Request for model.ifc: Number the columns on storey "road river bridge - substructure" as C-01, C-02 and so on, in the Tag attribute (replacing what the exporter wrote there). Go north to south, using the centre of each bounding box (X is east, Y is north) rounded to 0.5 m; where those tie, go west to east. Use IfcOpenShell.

First a look at what the model holds.

```python
import ifcopenshell
import ifcopenshell.util.element
import ifcopenshell.util.placement

model = ifcopenshell.open("model.ifc")
print(model.schema)
storey = next(s for s in model.by_type("IfcBuildingStorey") if s.Name == "road river bridge - substructure")
columns = [e for e in ifcopenshell.util.element.get_decomposition(storey) if e.is_a("IfcColumn")]
for e in sorted(columns, key=lambda e: e.id()):
    origin = ifcopenshell.util.placement.get_local_placement(e.ObjectPlacement)[:3, 3]
    print(e.id(), e.Tag, e.Name, origin.round(2) + 0.0, sep=" | ")
```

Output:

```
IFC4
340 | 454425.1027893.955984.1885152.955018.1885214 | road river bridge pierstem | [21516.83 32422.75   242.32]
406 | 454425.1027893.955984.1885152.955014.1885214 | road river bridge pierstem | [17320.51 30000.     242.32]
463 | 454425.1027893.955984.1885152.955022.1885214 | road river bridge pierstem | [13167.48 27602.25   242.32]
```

```python
import ifcopenshell
import ifcopenshell.geom
import ifcopenshell.util.element
import ifcopenshell.util.shape

model = ifcopenshell.open("model.ifc")
settings = ifcopenshell.geom.settings()
settings.set("use-world-coords", True)


def centre(element):
    shape = ifcopenshell.geom.create_shape(settings, element)
    return ifcopenshell.util.shape.get_bbox_centroid(shape.geometry)


storey = next(s for s in model.by_type("IfcBuildingStorey") if s.Name == "road river bridge - substructure")
columns = [e for e in ifcopenshell.util.element.get_decomposition(storey) if e.is_a("IfcColumn")]

# Insertion points can sit at a corner or the storey origin, so sort by the geometry (in metres).
centres = {e: centre(e) for e in columns}
columns.sort(key=lambda e: (-round(centres[e][1] / 0.5), centres[e][0]))

for i, e in enumerate(columns, start=1):
    number = f"C-{i:02d}"
    e.Tag = number
    print(e.id(), number)

model.write("model_v2.ifc")
```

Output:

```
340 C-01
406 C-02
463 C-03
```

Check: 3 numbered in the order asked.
